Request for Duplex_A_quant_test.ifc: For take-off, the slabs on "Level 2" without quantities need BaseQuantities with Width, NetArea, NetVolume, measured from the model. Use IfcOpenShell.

First a look at what the model holds.

```python
import ifcopenshell
import ifcopenshell.util.element
import ifcopenshell.util.unit

model = ifcopenshell.open("Duplex_A_quant_test.ifc")
print(model.schema)
for unit_type in ("LENGTHUNIT", "AREAUNIT", "VOLUMEUNIT"):
    print(unit_type, ifcopenshell.util.unit.calculate_unit_scale(model, unit_type))
storey = next(s for s in model.by_type("IfcBuildingStorey") if s.Name == "Level 2")
slabs = [e for e in ifcopenshell.util.element.get_decomposition(storey) if e.is_a("IfcSlab")]
for e in sorted(slabs, key=lambda e: e.id()):
    print(e.id(), e.is_a(), e.Name, list(ifcopenshell.util.element.get_psets(e, qtos_only=True)), sep=" | ")
```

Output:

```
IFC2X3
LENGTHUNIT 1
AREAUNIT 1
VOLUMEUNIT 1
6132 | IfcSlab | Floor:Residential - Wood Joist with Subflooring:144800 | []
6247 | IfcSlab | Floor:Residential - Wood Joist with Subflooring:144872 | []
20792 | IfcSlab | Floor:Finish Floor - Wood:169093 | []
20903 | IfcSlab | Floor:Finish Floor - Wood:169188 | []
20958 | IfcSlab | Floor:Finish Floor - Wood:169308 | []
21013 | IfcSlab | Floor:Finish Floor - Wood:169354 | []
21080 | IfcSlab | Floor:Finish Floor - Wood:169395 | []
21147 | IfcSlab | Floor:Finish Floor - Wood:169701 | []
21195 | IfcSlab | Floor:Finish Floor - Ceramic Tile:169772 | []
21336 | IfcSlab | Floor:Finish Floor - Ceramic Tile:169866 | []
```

```python
import ifcopenshell
import ifcopenshell.api.pset
import ifcopenshell.geom
import ifcopenshell.util.element
import ifcopenshell.util.shape
import ifcopenshell.util.unit

model = ifcopenshell.open("Duplex_A_quant_test.ifc")
unit_scale = ifcopenshell.util.unit.calculate_unit_scale(model)
area_scale = ifcopenshell.util.unit.calculate_unit_scale(model, "AREAUNIT")
volume_scale = ifcopenshell.util.unit.calculate_unit_scale(model, "VOLUMEUNIT")
settings = ifcopenshell.geom.settings()

storey = next(s for s in model.by_type("IfcBuildingStorey") if s.Name == "Level 2")
slabs = [e for e in ifcopenshell.util.element.get_decomposition(storey) if e.is_a("IfcSlab")]

for e in sorted(slabs, key=lambda e: e.id()):
    if ifcopenshell.util.element.get_psets(e, qtos_only=True, should_inherit=False):
        continue
    # Geometry comes back in metres, in the element's own axes.
    shape = ifcopenshell.geom.create_shape(settings, e)
    values = {
        "Width": ifcopenshell.util.shape.get_z(shape.geometry) / unit_scale,
        "NetArea": ifcopenshell.util.shape.get_footprint_area(shape.geometry) / area_scale,
        "NetVolume": ifcopenshell.util.shape.get_volume(shape.geometry) / volume_scale,
    }
    qto = ifcopenshell.api.pset.add_qto(model, product=e, name="BaseQuantities")
    ifcopenshell.api.pset.edit_qto(model, qto=qto, properties=values)
    print(e.id(), {k: round(v, 3) for k, v in values.items()})

model.write("Duplex_A_quant_test_updated.ifc")
```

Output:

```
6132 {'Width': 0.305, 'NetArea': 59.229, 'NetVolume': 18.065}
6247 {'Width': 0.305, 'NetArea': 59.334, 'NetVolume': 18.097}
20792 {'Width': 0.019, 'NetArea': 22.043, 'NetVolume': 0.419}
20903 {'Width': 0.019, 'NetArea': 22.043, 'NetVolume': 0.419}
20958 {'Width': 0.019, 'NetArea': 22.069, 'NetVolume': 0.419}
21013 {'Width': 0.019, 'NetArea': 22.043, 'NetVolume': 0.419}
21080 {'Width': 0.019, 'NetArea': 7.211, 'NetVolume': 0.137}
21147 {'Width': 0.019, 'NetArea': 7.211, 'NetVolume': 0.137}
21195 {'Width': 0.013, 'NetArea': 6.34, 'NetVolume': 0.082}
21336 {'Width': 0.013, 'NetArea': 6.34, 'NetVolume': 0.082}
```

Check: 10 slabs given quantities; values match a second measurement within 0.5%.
